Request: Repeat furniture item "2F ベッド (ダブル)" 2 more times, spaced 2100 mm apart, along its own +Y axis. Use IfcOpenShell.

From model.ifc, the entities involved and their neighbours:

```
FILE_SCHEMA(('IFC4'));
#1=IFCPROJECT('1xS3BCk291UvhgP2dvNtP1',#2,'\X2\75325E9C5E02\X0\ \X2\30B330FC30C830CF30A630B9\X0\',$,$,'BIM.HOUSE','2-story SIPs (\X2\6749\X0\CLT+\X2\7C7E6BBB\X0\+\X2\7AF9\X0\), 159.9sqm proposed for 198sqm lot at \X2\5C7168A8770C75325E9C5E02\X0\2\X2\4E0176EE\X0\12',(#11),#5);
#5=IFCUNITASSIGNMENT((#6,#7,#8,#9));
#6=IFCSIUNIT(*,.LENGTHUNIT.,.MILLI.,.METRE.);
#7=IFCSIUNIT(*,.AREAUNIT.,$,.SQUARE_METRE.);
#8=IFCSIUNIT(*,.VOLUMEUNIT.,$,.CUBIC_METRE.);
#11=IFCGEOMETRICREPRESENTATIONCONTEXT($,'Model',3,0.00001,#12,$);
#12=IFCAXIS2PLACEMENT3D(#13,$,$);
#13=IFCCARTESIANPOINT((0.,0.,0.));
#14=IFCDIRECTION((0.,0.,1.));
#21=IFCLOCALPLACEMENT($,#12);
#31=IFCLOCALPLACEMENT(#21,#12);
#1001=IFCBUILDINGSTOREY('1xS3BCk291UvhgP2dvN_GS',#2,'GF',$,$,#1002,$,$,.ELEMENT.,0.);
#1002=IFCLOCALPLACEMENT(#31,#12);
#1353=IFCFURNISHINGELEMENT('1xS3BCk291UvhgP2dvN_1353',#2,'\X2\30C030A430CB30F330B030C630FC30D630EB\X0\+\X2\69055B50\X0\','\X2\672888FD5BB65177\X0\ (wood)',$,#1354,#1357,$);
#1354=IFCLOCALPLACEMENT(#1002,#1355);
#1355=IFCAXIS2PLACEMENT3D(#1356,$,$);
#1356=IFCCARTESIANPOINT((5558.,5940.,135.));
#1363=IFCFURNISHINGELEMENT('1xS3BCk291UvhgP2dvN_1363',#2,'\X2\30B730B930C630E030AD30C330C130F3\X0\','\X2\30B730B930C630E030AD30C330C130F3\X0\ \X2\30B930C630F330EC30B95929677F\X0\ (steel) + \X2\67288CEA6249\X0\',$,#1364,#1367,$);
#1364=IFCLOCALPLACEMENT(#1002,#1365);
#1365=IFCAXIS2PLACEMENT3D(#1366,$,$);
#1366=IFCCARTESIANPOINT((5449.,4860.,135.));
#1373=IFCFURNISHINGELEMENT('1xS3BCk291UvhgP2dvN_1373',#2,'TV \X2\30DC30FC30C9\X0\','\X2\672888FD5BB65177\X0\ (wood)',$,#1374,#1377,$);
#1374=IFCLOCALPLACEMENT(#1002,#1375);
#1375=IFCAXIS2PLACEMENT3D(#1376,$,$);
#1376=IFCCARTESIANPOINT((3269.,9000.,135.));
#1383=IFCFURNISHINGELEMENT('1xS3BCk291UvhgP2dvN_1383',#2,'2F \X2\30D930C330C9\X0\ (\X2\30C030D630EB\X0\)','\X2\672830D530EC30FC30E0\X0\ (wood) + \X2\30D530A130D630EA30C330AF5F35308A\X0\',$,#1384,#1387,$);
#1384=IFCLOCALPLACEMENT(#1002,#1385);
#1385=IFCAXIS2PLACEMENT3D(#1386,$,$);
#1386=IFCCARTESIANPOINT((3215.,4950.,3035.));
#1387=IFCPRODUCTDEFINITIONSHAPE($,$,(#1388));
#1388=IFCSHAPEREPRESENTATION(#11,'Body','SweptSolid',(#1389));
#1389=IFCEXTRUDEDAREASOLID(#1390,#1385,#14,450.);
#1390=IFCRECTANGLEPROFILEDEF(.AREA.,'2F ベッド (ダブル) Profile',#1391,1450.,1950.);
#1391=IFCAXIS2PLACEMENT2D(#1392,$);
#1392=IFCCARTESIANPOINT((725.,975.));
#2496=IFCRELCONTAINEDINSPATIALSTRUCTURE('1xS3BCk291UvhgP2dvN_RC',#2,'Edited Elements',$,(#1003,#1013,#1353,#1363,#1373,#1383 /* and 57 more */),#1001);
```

```python
import ifcopenshell
import ifcopenshell.api.geometry
import ifcopenshell.api.root
import ifcopenshell.util.element
import ifcopenshell.util.placement
import ifcopenshell.util.unit

model = ifcopenshell.open("model.ifc")
unit_scale = ifcopenshell.util.unit.calculate_unit_scale(model)


def reuse_history(source, copy):
    """copy_class also copies each property set's owner history, people and application; keep the originals."""
    for rel in copy.IsDefinedBy:
        if rel.is_a("IfcRelDefinesByProperties") and (history := rel.RelatingPropertyDefinition.OwnerHistory):
            rel.RelatingPropertyDefinition.OwnerHistory = source.OwnerHistory
            ifcopenshell.util.element.remove_deep2(model, history)


source = model.by_guid("1xS3BCk291UvhgP2dvN_1383")
base = ifcopenshell.util.placement.get_local_placement(source.ObjectPlacement)
step = base[:3, 1] * 2.1 / unit_scale

for i in range(1, 3):
    copy = ifcopenshell.api.root.copy_class(model, product=source)
    copy.Representation = ifcopenshell.util.element.copy_deep(
        model, source.Representation, exclude=["IfcGeometricRepresentationContext", "IfcRepresentationMap"]
    )
    reuse_history(source, copy)
    matrix = base.copy()
    matrix[:3, 3] += i * step
    print("added at", matrix[:3, 3].round(3) + 0.0)
    ifcopenshell.api.geometry.edit_object_placement(model, product=copy, matrix=matrix, is_si=False)

model.write("model-out.ifc")
```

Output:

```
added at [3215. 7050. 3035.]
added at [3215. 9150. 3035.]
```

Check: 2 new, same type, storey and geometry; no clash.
